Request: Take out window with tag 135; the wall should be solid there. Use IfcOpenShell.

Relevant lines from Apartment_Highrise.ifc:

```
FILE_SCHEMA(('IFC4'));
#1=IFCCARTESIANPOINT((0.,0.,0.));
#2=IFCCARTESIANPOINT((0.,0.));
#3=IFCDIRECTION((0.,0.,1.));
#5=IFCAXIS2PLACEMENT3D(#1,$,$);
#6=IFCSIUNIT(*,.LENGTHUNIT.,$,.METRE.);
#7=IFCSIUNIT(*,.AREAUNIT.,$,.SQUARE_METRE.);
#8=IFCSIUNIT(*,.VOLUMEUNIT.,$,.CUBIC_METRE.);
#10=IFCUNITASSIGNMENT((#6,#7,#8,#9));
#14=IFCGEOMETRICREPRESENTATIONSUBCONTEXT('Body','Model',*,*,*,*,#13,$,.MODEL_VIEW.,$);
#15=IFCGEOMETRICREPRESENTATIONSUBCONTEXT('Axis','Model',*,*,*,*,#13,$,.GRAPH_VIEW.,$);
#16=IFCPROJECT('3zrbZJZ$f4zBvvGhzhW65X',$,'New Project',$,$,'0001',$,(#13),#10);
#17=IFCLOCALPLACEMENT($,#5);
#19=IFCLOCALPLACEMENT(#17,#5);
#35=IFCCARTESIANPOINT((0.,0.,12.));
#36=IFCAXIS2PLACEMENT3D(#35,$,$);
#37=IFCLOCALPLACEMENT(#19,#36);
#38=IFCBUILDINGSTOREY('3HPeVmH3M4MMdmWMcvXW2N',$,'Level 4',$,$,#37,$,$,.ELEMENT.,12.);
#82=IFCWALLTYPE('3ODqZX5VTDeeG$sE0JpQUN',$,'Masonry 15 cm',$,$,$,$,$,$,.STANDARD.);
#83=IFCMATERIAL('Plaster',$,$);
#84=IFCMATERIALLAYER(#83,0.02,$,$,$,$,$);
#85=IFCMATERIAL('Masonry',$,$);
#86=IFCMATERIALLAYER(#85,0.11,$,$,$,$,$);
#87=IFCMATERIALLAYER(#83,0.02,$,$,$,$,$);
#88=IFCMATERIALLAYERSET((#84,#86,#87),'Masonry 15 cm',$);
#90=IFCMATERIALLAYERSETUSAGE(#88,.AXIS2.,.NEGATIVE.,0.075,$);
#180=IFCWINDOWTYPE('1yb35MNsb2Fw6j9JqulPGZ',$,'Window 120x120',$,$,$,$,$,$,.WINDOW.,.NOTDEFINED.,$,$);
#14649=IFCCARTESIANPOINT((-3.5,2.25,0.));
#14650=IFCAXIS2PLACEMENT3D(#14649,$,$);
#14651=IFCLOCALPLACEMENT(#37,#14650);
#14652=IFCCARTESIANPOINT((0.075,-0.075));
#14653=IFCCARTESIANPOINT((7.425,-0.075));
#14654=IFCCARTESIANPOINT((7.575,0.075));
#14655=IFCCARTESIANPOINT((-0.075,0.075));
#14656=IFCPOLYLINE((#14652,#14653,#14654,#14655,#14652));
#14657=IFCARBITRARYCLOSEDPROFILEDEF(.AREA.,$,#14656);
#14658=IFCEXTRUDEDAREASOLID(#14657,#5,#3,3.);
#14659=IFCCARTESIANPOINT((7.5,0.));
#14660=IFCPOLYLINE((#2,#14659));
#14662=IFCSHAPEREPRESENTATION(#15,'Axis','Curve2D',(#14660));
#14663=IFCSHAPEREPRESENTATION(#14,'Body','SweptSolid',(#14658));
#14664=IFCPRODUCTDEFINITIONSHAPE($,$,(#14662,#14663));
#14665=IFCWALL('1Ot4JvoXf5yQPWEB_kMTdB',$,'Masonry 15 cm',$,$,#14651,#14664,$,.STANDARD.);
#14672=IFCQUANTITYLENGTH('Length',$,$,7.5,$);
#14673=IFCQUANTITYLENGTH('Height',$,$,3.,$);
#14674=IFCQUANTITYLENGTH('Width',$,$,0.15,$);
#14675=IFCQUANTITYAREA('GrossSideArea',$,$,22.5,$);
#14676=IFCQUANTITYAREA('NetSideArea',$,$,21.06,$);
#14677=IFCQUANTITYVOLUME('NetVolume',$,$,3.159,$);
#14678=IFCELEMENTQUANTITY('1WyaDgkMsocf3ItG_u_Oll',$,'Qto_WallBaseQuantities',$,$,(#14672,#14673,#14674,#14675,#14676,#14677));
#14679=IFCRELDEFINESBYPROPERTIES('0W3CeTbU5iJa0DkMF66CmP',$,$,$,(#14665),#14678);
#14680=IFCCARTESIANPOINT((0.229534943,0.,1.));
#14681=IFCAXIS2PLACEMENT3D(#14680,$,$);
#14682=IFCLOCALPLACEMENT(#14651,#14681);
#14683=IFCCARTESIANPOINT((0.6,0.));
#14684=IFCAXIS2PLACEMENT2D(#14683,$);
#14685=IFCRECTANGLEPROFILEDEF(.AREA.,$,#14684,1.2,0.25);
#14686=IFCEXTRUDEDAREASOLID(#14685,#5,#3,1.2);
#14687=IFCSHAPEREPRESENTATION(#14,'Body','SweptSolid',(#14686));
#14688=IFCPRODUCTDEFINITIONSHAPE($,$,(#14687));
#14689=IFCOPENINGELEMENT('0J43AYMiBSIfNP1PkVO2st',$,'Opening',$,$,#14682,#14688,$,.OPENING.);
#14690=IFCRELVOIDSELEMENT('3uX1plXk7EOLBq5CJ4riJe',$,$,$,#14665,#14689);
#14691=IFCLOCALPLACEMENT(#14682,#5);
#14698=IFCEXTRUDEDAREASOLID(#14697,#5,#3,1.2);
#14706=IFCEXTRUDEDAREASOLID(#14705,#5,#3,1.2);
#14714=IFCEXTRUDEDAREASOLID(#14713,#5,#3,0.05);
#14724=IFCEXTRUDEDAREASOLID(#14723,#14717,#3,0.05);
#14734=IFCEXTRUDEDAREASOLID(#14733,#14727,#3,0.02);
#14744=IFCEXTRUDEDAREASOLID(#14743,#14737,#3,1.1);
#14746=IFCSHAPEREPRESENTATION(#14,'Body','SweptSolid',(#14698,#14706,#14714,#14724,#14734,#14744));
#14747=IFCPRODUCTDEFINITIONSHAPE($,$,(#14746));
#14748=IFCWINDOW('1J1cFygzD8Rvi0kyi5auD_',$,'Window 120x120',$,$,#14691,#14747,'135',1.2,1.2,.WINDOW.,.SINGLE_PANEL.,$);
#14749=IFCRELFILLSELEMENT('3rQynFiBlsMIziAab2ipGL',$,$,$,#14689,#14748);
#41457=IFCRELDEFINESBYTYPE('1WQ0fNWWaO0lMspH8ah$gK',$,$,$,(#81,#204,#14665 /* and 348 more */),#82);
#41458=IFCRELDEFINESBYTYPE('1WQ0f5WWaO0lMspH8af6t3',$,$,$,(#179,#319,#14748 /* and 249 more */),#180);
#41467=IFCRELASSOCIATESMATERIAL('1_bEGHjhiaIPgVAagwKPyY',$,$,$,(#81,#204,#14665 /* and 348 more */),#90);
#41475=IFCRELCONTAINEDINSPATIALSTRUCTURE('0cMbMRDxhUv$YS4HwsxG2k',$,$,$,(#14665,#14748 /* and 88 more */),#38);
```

```python
import ifcopenshell
import ifcopenshell.api.feature
import ifcopenshell.api.pset
import ifcopenshell.api.root
import ifcopenshell.geom
import ifcopenshell.util.element
import ifcopenshell.util.shape
import ifcopenshell.util.unit

model = ifcopenshell.open("Apartment_Highrise.ifc")
area_scale = ifcopenshell.util.unit.calculate_unit_scale(model, "AREAUNIT")
volume_scale = ifcopenshell.util.unit.calculate_unit_scale(model, "VOLUMEUNIT")
settings = ifcopenshell.geom.settings()


def volume(element):
    """Net volume in cubic metres, openings subtracted."""
    shape = ifcopenshell.geom.create_shape(settings, element)
    return ifcopenshell.util.shape.get_volume(shape.geometry)


window = model.by_guid("1J1cFygzD8Rvi0kyi5auD_")
opening = window.FillsVoids[0].RelatingOpeningElement
wall = opening.VoidsElements[0].RelatingBuildingElement
before = volume(wall)

ifcopenshell.api.root.remove_product(model, product=window)
ifcopenshell.api.feature.remove_feature(model, feature=opening)

after = volume(wall)
thickness = 0.15  # wall thickness in metres

# Update the wall's stored quantities.
qto = model.by_id(ifcopenshell.util.element.get_pset(wall, "Qto_WallBaseQuantities", should_inherit=False)["id"])
ifcopenshell.api.pset.edit_qto(model, qto=qto, properties={
    "NetSideArea": after / thickness / area_scale,
    "NetVolume": after / volume_scale,
})

print(f"wall volume {before:.3f} -> {after:.3f} m3")

model.write("Apartment_Highrise_updated.ifc")
```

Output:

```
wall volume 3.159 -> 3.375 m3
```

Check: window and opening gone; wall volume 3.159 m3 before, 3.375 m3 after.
